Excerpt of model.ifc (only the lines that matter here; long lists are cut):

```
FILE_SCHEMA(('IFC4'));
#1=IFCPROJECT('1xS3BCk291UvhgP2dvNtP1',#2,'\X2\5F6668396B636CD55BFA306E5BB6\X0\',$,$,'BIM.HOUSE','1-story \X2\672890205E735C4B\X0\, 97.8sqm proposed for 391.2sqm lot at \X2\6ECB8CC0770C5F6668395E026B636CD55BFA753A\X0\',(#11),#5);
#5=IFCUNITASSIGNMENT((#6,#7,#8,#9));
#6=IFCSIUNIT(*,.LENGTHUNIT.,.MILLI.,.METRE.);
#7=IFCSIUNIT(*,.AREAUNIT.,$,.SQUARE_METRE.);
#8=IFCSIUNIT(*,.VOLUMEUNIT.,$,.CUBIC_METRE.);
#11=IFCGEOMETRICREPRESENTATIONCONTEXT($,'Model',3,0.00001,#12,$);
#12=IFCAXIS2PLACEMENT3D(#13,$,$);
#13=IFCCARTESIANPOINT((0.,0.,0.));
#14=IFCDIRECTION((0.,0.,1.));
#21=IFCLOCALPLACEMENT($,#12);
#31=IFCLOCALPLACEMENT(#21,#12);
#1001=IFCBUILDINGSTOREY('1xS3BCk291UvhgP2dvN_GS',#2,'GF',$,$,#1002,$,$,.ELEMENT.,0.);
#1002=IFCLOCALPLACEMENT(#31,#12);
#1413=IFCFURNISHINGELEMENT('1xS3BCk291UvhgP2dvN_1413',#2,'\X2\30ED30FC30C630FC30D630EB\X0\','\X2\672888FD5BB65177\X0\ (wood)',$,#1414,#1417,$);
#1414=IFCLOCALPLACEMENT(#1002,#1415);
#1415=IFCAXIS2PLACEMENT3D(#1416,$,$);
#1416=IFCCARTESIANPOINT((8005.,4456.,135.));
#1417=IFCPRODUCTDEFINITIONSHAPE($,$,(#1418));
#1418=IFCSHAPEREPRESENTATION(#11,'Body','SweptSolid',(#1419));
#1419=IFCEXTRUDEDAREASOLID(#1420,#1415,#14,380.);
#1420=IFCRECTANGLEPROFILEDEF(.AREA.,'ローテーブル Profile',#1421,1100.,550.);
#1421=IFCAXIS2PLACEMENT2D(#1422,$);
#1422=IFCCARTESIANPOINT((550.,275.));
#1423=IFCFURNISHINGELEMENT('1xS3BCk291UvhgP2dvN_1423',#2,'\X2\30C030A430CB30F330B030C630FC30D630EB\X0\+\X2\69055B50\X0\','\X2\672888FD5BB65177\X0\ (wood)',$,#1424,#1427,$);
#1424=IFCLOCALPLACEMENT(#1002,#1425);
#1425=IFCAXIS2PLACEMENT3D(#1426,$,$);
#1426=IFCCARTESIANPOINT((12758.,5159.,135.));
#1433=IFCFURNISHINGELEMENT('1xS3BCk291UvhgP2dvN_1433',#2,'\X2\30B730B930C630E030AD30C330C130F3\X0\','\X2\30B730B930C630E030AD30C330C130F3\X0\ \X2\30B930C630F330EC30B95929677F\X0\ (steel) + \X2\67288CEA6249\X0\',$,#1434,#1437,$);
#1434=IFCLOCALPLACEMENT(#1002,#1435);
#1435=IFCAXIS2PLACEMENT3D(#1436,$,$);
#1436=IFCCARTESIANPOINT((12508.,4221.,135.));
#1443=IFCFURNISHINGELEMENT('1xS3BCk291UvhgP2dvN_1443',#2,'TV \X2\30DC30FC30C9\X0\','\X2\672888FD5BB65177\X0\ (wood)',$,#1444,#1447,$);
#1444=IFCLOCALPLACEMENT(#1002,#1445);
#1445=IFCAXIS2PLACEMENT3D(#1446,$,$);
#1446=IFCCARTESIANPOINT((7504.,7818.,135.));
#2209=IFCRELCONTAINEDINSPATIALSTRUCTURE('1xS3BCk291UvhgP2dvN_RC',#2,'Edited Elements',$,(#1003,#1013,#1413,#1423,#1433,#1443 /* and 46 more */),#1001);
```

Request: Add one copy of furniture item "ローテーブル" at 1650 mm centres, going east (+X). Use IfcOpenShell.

```python
import numpy as np
import ifcopenshell
import ifcopenshell.api.geometry
import ifcopenshell.api.root
import ifcopenshell.util.element
import ifcopenshell.util.placement

model = ifcopenshell.open("model.ifc")


def reuse_history(source, copy):
    """copy_class also copies each property set's owner history, people and application; keep the originals."""
    for rel in copy.IsDefinedBy:
        if rel.is_a("IfcRelDefinesByProperties") and (history := rel.RelatingPropertyDefinition.OwnerHistory):
            rel.RelatingPropertyDefinition.OwnerHistory = source.OwnerHistory
            ifcopenshell.util.element.remove_deep2(model, history)


source = model.by_id(1413)
base = ifcopenshell.util.placement.get_local_placement(source.ObjectPlacement)
step = np.array([1.0, 0.0, 0.0]) * 1650.0

for i in range(1, 2):
    copy = ifcopenshell.api.root.copy_class(model, product=source)
    copy.Representation = ifcopenshell.util.element.copy_deep(
        model, source.Representation, exclude=["IfcGeometricRepresentationContext", "IfcRepresentationMap"]
    )
    reuse_history(source, copy)
    matrix = base.copy()
    matrix[:3, 3] += i * step
    print("added at", matrix[:3, 3].round(3) + 0.0)
    ifcopenshell.api.geometry.edit_object_placement(model, product=copy, matrix=matrix, is_si=False)

model.write("model_rev.ifc")
```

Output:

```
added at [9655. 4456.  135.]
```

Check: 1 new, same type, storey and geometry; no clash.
